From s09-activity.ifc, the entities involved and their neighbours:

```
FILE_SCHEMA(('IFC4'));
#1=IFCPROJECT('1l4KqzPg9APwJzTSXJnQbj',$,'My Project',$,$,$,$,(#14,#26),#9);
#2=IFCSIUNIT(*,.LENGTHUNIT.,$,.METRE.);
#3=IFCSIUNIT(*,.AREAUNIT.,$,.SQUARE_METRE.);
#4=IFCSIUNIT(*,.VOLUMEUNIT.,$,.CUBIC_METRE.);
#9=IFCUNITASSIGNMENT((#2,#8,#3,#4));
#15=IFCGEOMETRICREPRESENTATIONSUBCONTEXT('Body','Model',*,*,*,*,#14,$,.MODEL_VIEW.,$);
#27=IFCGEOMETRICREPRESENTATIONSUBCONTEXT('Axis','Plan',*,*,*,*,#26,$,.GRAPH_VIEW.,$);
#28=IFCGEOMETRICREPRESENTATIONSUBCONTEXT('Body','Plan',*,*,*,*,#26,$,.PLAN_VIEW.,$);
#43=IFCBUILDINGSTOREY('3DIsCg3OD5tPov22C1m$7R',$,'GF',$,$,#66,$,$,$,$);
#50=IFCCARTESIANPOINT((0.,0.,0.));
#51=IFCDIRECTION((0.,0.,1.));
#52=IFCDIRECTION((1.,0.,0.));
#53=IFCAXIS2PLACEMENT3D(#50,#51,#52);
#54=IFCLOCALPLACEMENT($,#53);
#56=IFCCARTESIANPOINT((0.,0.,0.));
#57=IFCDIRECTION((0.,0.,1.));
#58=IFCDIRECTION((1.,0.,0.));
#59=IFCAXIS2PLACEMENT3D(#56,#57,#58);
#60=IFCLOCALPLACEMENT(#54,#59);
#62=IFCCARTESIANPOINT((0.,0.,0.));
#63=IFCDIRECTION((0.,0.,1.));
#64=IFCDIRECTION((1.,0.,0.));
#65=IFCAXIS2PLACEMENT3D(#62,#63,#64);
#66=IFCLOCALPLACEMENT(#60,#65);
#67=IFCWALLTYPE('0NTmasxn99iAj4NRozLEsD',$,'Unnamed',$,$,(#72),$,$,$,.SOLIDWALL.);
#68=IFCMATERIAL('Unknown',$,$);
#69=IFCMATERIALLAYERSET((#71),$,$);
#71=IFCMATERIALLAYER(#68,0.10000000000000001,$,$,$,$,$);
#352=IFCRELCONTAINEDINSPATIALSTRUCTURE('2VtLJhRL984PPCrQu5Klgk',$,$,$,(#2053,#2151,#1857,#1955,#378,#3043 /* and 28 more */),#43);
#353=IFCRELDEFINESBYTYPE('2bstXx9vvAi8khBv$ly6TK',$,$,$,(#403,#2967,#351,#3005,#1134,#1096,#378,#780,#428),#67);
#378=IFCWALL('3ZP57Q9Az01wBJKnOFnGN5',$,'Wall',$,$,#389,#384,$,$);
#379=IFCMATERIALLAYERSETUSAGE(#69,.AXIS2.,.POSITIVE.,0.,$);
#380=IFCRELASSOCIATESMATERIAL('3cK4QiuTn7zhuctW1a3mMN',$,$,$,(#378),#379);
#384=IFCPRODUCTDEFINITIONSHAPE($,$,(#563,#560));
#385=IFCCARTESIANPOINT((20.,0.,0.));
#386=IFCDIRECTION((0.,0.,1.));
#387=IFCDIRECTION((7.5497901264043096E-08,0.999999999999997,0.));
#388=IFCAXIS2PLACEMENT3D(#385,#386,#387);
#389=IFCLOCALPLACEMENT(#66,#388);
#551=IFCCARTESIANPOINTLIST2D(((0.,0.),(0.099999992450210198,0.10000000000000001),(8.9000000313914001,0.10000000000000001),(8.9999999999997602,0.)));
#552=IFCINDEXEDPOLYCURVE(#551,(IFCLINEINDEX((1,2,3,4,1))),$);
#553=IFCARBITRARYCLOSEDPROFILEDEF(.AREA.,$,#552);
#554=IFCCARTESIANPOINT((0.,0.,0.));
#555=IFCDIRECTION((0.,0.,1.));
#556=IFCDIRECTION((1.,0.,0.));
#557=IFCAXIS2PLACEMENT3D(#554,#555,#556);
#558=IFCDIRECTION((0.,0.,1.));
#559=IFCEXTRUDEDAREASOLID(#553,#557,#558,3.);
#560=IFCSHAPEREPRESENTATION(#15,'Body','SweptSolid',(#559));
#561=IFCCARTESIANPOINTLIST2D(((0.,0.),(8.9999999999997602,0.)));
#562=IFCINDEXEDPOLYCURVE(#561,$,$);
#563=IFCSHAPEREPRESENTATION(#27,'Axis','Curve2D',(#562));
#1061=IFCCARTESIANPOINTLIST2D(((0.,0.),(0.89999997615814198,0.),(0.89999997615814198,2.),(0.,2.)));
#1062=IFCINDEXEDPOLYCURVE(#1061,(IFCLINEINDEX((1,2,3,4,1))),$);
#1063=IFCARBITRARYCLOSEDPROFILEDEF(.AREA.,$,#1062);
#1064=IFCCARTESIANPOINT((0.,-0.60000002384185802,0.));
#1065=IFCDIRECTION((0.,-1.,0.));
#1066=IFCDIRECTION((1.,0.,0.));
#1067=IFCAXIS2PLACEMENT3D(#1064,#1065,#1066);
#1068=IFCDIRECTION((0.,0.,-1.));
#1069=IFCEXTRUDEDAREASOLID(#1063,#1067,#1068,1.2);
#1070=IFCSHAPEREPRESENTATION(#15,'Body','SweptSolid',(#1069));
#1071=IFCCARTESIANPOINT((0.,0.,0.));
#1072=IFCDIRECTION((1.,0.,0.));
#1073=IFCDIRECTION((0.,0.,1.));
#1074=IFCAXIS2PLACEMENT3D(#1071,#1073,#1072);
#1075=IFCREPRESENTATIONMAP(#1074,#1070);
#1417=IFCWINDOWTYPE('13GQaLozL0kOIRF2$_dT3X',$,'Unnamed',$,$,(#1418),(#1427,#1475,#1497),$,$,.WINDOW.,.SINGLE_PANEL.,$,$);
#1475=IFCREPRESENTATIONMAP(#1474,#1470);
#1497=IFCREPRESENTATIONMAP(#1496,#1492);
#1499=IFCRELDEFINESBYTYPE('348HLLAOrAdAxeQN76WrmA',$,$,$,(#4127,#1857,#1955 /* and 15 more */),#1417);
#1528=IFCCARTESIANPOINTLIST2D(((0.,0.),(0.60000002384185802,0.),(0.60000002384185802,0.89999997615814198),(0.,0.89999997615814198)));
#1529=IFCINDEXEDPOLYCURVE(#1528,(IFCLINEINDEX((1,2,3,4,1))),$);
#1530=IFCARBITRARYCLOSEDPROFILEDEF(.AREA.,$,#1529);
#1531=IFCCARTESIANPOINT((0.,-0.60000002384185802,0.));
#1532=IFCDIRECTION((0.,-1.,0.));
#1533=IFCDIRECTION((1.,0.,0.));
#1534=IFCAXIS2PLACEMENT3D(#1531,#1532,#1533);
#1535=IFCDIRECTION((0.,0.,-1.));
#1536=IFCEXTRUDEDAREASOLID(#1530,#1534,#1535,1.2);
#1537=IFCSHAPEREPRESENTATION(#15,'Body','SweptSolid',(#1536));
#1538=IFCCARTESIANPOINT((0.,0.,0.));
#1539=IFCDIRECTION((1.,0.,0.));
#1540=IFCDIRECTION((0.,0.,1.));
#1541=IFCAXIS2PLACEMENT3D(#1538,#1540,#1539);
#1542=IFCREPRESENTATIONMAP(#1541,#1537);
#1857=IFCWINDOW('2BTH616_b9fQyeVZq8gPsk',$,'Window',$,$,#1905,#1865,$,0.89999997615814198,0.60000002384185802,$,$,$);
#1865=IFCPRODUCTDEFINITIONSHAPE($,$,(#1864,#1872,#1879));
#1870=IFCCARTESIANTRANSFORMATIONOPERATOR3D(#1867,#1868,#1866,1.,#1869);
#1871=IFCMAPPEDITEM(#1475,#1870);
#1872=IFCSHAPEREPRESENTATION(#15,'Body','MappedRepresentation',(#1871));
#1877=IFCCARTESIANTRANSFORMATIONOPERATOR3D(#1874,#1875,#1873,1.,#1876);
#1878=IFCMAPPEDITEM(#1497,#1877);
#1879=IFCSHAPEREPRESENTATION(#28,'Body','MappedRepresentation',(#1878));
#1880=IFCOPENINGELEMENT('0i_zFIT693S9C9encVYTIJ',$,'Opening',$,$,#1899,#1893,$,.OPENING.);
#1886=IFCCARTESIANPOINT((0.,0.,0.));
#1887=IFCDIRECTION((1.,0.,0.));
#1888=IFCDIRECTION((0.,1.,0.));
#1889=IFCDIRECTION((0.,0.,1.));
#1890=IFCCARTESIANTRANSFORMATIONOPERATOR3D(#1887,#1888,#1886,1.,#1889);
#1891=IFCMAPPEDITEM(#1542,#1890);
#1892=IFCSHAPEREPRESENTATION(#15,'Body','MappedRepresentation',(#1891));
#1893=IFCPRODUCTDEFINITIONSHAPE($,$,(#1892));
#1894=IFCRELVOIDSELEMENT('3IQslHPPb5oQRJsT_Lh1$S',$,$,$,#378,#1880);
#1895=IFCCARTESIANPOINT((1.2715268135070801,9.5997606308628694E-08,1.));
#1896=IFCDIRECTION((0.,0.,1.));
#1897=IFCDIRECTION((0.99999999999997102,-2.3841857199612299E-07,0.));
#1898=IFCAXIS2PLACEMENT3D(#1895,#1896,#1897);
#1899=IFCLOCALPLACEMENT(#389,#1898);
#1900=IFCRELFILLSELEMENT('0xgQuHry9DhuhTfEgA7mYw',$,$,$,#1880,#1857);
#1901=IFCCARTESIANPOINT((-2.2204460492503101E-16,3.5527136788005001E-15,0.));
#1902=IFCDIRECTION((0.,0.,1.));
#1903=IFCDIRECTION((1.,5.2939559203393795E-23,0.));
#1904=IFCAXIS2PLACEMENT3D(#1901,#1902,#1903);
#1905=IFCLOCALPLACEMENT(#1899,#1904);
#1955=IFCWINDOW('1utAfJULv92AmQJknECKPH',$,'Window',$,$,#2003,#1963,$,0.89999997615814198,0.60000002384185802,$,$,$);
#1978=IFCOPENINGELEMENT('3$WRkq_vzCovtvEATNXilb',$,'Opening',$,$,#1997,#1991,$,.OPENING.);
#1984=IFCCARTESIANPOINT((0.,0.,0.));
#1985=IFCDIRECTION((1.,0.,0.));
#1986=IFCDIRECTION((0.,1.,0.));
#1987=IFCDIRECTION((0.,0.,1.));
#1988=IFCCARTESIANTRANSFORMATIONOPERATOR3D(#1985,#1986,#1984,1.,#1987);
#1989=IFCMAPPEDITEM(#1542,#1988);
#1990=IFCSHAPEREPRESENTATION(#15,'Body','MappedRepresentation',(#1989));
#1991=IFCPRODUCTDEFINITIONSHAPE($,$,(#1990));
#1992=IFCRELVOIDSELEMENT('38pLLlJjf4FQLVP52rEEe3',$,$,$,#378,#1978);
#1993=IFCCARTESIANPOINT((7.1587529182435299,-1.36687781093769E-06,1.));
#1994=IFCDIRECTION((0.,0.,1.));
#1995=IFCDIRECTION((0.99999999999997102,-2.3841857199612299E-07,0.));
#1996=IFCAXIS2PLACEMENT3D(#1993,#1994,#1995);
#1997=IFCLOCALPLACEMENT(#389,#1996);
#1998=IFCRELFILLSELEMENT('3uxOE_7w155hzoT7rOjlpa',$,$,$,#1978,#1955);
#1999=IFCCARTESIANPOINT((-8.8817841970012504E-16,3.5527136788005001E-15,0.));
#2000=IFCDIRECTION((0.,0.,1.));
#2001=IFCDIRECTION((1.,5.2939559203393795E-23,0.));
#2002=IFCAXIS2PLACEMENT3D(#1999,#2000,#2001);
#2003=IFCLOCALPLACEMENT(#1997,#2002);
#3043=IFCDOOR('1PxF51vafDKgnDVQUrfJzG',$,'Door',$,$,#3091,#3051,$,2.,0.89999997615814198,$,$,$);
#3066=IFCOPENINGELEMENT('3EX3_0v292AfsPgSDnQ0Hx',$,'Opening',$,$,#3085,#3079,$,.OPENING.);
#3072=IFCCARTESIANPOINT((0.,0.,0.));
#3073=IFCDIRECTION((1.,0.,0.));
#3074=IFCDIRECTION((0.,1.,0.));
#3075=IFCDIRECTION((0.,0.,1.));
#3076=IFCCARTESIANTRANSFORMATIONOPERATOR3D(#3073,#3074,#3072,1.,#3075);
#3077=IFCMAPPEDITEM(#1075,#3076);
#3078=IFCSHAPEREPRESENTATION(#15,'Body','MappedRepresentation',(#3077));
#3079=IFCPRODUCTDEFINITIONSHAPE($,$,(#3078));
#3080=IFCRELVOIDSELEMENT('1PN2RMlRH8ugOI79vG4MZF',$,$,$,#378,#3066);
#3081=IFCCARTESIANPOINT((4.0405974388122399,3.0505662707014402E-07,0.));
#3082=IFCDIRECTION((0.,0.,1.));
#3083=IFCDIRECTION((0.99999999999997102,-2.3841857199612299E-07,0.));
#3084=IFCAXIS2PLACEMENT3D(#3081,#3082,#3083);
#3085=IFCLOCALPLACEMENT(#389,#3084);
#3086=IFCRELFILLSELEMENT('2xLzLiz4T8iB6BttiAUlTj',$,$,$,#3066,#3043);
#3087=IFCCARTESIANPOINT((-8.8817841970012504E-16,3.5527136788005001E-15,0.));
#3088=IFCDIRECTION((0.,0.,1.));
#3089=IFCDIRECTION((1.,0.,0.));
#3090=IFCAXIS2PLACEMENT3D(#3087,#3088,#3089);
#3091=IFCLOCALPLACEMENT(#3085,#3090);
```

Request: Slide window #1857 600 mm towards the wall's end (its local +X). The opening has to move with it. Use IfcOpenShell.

```python
import ifcopenshell
import ifcopenshell.api.geometry
import ifcopenshell.util.placement
import ifcopenshell.util.unit

model = ifcopenshell.open("s09-activity.ifc")
unit_scale = ifcopenshell.util.unit.calculate_unit_scale(model)

window = model.by_guid("2BTH616_b9fQyeVZq8gPsk")
opening = window.FillsVoids[0].RelatingOpeningElement
wall = opening.VoidsElements[0].RelatingBuildingElement

wall_matrix = ifcopenshell.util.placement.get_local_placement(wall.ObjectPlacement)
shift = wall_matrix[:3, 0] * 0.6 / unit_scale
before = ifcopenshell.util.placement.get_local_placement(window.ObjectPlacement)[:3, 3].copy()

# The window is placed relative to its opening, so it follows when the opening moves.
matrix = ifcopenshell.util.placement.get_local_placement(opening.ObjectPlacement)
matrix[:3, 3] += shift
ifcopenshell.api.geometry.edit_object_placement(
    model, product=opening, matrix=matrix, is_si=False, should_transform_children=True
)

after = ifcopenshell.util.placement.get_local_placement(window.ObjectPlacement)[:3, 3]
print("window moved by", (after - before).round(3) + 0.0)

model.write("s09-activity_edited.ifc")
```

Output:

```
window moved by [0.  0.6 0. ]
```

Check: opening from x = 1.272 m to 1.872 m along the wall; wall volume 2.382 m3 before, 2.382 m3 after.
